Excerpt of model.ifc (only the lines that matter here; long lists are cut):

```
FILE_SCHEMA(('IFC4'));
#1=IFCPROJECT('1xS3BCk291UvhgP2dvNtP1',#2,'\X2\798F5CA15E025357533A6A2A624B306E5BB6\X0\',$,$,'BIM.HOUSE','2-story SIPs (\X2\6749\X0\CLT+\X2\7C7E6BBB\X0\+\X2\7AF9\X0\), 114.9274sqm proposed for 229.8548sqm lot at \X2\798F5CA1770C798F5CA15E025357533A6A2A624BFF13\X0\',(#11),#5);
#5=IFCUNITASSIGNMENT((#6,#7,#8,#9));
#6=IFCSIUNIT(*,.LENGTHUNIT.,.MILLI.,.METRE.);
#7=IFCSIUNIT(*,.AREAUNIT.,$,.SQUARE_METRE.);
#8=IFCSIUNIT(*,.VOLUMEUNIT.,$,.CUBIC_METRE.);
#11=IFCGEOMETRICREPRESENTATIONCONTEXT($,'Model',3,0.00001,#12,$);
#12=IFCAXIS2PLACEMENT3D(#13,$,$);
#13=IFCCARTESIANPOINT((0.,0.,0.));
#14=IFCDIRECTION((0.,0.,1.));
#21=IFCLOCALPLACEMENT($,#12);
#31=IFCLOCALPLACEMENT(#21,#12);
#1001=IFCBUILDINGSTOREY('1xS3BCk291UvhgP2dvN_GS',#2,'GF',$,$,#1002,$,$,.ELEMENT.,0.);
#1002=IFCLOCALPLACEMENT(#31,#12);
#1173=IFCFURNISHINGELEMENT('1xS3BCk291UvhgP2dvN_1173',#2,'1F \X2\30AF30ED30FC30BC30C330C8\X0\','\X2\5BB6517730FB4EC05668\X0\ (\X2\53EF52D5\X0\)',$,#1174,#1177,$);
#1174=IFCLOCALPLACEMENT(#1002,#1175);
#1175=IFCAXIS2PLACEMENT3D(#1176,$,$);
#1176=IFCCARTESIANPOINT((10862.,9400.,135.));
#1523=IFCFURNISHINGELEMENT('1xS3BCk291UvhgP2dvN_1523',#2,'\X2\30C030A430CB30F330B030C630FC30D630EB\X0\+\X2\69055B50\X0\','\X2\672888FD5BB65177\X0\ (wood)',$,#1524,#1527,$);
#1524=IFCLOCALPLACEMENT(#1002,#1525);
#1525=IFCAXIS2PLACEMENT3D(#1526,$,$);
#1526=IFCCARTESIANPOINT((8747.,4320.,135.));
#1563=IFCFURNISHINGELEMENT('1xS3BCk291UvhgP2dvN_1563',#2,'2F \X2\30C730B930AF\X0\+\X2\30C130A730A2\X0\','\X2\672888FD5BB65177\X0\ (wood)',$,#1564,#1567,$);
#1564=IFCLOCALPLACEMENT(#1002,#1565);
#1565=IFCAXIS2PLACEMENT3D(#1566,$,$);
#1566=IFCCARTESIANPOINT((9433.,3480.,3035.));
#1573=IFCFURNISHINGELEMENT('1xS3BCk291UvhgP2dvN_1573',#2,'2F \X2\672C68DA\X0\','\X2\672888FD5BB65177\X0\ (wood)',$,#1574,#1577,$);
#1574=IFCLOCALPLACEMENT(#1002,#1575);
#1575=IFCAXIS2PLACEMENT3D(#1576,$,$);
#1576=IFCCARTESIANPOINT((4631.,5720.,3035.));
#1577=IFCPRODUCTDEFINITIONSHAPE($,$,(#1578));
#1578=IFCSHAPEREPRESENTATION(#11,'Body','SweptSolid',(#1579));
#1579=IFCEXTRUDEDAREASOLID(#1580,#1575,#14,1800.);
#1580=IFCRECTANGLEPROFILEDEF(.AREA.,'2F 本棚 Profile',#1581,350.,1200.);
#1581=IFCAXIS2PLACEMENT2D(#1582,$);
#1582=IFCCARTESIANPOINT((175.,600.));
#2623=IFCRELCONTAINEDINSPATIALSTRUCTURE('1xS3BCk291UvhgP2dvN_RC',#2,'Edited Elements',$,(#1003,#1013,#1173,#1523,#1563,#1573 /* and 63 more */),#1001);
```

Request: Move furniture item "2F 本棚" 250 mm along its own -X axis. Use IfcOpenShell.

```python
import ifcopenshell
import ifcopenshell.api.geometry
import ifcopenshell.util.placement

model = ifcopenshell.open("model.ifc")

item = model.by_id(1573)
matrix = ifcopenshell.util.placement.get_local_placement(item.ObjectPlacement)
matrix[:3, 3] -= matrix[:3, 0] * 250.0
ifcopenshell.api.geometry.edit_object_placement(model, product=item, matrix=matrix, is_si=False)

print(ifcopenshell.util.placement.get_local_placement(item.ObjectPlacement).round(3) + 0.0)

model.write("model_rev.ifc")
```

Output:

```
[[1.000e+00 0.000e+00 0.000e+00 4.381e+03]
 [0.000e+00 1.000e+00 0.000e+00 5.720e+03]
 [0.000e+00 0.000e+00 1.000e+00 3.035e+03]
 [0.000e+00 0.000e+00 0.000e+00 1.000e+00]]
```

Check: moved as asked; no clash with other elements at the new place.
